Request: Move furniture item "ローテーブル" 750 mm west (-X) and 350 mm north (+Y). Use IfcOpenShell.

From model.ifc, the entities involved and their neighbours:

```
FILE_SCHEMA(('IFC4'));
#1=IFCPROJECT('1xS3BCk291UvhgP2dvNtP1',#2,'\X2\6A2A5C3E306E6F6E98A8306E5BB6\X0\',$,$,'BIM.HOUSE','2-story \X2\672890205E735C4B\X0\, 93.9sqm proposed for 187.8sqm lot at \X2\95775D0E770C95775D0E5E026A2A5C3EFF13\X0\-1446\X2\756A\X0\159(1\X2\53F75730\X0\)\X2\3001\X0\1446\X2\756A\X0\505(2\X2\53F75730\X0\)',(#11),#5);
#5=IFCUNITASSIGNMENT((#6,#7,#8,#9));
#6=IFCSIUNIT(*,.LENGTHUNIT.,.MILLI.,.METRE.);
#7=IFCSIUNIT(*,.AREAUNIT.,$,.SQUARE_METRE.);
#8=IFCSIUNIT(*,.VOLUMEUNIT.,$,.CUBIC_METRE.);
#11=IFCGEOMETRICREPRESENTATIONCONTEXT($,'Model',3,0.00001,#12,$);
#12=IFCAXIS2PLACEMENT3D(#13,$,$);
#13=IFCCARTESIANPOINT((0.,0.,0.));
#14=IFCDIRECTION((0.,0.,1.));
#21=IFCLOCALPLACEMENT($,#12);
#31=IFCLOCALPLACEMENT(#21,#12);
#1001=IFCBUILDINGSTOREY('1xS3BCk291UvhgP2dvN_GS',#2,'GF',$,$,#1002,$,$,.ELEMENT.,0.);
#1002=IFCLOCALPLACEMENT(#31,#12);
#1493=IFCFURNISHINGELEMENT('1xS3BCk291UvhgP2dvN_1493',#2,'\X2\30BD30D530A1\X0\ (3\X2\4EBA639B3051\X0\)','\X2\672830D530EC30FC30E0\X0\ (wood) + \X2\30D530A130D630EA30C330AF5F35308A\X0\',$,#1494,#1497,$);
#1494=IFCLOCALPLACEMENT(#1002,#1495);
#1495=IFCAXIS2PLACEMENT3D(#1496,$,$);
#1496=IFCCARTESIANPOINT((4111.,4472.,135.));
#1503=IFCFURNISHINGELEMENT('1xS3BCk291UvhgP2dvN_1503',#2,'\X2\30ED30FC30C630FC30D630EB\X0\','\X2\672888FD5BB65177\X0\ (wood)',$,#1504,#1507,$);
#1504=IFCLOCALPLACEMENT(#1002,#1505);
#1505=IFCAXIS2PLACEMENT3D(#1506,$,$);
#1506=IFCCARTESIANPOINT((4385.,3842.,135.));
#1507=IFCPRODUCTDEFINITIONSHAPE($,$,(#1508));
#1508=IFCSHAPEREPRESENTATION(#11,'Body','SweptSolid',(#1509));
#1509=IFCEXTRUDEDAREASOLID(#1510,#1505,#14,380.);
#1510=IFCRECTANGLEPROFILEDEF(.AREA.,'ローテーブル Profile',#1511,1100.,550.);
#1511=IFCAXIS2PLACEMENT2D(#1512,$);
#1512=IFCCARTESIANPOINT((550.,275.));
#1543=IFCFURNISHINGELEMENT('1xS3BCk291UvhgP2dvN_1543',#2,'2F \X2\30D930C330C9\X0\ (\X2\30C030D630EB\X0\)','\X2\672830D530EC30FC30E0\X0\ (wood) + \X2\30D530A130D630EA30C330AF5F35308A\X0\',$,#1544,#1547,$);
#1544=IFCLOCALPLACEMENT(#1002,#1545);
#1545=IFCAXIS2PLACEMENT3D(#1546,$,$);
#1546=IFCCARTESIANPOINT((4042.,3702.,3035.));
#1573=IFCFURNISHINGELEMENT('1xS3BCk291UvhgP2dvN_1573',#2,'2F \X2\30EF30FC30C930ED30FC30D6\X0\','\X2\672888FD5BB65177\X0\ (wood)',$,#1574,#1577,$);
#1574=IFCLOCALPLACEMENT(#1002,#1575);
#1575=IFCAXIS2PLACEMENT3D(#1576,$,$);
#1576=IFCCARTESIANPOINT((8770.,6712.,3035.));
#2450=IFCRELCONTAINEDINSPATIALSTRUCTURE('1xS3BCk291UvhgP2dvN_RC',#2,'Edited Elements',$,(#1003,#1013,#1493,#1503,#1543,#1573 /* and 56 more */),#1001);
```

```python
import ifcopenshell
import ifcopenshell.api.geometry
import ifcopenshell.util.placement
import ifcopenshell.util.unit

model = ifcopenshell.open("model.ifc")
unit_scale = ifcopenshell.util.unit.calculate_unit_scale(model)

item = model.by_id(1503)
matrix = ifcopenshell.util.placement.get_local_placement(item.ObjectPlacement)
matrix[0, 3] -= 0.75 / unit_scale
matrix[1, 3] += 0.35 / unit_scale
ifcopenshell.api.geometry.edit_object_placement(model, product=item, matrix=matrix, is_si=False)

print(ifcopenshell.util.placement.get_local_placement(item.ObjectPlacement).round(3) + 0.0)

model.write("model_edited.ifc")
```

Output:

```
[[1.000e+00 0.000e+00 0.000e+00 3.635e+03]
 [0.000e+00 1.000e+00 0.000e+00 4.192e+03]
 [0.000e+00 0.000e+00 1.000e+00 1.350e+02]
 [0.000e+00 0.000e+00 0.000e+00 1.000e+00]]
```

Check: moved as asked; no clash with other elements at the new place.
